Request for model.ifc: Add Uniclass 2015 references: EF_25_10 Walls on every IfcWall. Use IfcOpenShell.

First a look at what the model holds.

```python
import ifcopenshell

model = ifcopenshell.open("model.ifc")
print(model.schema)
print("classifications:", [c.Name for c in model.by_type("IfcClassification")])
for ifc_class in ("IfcDoor", "IfcRoof", "IfcStair", "IfcWall", "IfcWindow"):
    print(ifc_class, len(model.by_type(ifc_class)))
```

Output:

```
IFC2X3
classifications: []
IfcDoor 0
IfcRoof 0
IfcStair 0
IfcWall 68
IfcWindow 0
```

```python
import ifcopenshell
import ifcopenshell.api.classification

model = ifcopenshell.open("model.ifc")

# IFC2X3 requires Source and Edition and has no link from the project to the system.
system = model.create_entity("IfcClassification", Source="NBS", Edition="2015", Name="Uniclass 2015")

codes = {
    "IfcWall": ("EF_25_10", "Walls"),
}
for ifc_class, (code, name) in codes.items():
    products = model.by_type(ifc_class)
    ifcopenshell.api.classification.add_reference(
        model, products=products, classification=system, identification=code, name=name
    )
    print(code, len(products))

model.write("model_rev.ifc")
```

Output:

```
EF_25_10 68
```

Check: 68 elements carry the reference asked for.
